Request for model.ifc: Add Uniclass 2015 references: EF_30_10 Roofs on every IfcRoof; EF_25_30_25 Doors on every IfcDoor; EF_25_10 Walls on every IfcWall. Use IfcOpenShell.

First a look at what the model holds.

```python
import ifcopenshell

model = ifcopenshell.open("model.ifc")
print(model.schema)
print("classifications:", [c.Name for c in model.by_type("IfcClassification")])
for ifc_class in ("IfcDoor", "IfcRoof", "IfcStair", "IfcWall", "IfcWindow"):
    print(ifc_class, len(model.by_type(ifc_class)))
```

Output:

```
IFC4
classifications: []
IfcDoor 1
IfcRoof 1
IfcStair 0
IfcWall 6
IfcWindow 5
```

```python
import ifcopenshell
import ifcopenshell.api.classification

model = ifcopenshell.open("model.ifc")

system = ifcopenshell.api.classification.add_classification(model, classification="Uniclass 2015")

codes = {
    "IfcRoof": ("EF_30_10", "Roofs"),
    "IfcDoor": ("EF_25_30_25", "Doors"),
    "IfcWall": ("EF_25_10", "Walls"),
}
for ifc_class, (code, name) in codes.items():
    products = model.by_type(ifc_class)
    ifcopenshell.api.classification.add_reference(
        model, products=products, classification=system, identification=code, name=name
    )
    print(code, len(products))

model.write("model-out.ifc")
```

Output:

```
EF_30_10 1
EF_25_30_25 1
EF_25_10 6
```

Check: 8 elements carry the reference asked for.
